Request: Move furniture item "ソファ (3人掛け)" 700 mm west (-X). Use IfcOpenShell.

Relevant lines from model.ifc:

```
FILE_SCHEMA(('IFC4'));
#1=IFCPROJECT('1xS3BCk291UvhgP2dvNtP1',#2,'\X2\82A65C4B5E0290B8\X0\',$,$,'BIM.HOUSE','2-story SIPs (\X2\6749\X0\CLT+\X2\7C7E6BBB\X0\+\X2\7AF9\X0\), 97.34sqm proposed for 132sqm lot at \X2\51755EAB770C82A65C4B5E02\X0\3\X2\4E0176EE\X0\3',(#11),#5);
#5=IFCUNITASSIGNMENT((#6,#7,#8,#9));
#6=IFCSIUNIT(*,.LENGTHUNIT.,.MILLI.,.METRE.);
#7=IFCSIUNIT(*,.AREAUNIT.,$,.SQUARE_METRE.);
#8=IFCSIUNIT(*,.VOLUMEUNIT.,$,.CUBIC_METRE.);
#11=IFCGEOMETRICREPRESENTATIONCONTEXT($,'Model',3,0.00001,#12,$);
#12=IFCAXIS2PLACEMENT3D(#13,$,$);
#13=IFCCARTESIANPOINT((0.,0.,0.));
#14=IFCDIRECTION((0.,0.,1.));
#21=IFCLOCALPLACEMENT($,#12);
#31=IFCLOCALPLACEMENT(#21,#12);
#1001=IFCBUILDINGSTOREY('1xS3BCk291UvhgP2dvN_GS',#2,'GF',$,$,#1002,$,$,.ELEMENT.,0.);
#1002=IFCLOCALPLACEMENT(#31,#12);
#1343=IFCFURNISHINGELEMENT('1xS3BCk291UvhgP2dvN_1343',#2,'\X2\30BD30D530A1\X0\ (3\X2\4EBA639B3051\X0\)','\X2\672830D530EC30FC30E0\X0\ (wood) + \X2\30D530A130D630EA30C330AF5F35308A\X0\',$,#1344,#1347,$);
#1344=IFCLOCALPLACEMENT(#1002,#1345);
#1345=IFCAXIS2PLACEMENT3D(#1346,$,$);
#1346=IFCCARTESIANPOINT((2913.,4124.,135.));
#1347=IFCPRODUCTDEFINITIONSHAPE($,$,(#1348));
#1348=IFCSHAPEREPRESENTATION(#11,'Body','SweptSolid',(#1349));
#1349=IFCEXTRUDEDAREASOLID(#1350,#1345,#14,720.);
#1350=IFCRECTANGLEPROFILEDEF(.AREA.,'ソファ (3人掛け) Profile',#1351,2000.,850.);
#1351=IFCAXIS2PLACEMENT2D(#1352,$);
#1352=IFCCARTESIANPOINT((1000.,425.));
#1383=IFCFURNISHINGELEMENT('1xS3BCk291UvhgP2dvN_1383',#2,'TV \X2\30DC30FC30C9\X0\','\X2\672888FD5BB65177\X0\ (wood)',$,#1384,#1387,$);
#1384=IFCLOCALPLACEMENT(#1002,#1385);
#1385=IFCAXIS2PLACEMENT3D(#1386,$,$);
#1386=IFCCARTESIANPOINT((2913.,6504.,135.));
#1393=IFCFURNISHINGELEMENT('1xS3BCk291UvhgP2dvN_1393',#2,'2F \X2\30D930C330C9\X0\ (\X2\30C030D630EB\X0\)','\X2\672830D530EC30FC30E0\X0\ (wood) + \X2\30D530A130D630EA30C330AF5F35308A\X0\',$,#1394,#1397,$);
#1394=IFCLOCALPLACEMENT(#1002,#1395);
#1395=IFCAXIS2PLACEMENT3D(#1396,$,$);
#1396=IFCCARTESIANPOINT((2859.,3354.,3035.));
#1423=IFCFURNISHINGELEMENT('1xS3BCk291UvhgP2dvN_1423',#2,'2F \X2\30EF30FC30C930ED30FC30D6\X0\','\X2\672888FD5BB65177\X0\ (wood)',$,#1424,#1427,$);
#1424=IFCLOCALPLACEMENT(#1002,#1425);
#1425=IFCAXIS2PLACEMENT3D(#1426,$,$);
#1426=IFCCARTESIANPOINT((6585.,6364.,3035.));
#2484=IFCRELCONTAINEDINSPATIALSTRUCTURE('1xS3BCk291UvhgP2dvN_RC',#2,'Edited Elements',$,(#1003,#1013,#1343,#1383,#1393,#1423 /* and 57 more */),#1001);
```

```python
import ifcopenshell
import ifcopenshell.api.geometry
import ifcopenshell.util.placement

model = ifcopenshell.open("model.ifc")

item = model.by_id(1343)
matrix = ifcopenshell.util.placement.get_local_placement(item.ObjectPlacement)
matrix[0, 3] -= 700.0
ifcopenshell.api.geometry.edit_object_placement(model, product=item, matrix=matrix, is_si=False)

print(ifcopenshell.util.placement.get_local_placement(item.ObjectPlacement).round(3) + 0.0)

model.write("model-out.ifc")
```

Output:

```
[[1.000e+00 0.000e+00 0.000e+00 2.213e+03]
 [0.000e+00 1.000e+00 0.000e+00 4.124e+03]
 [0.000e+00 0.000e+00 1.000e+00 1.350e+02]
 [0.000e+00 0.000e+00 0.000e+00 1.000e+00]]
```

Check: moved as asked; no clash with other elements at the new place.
